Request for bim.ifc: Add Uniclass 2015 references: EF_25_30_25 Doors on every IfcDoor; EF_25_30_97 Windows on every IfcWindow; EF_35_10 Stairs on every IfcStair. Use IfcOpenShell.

First a look at what the model holds.

```python
import ifcopenshell

model = ifcopenshell.open("bim.ifc")
print(model.schema)
print("classifications:", [c.Name for c in model.by_type("IfcClassification")])
for ifc_class in ("IfcDoor", "IfcRoof", "IfcStair", "IfcWall", "IfcWindow"):
    print(ifc_class, len(model.by_type(ifc_class)))
```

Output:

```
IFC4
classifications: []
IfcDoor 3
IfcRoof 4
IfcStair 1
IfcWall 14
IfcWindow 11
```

```python
import ifcopenshell
import ifcopenshell.api.classification

model = ifcopenshell.open("bim.ifc")

system = ifcopenshell.api.classification.add_classification(model, classification="Uniclass 2015")

codes = {
    "IfcDoor": ("EF_25_30_25", "Doors"),
    "IfcWindow": ("EF_25_30_97", "Windows"),
    "IfcStair": ("EF_35_10", "Stairs"),
}
for ifc_class, (code, name) in codes.items():
    products = model.by_type(ifc_class)
    ifcopenshell.api.classification.add_reference(
        model, products=products, classification=system, identification=code, name=name
    )
    print(code, len(products))

model.write("bim_rev.ifc")
```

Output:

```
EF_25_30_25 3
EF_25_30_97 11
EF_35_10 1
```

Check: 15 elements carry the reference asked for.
